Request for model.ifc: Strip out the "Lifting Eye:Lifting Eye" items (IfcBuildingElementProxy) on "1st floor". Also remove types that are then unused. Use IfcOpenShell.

First a look at what the model holds.

```python
import ifcopenshell
import ifcopenshell.util.element

model = ifcopenshell.open("model.ifc")
print(model.schema)
storey = next(s for s in model.by_type("IfcBuildingStorey") if s.Name == "1st floor")
proxies = [e for e in ifcopenshell.util.element.get_decomposition(storey) if e.is_a("IfcBuildingElementProxy")]
seen = {}
for e in proxies:
    element_type = ifcopenshell.util.element.get_type(e)
    name = element_type.Name if element_type not in (None, e) else None
    seen[name] = seen.get(name, 0) + 1
for name, count in sorted(seen.items(), key=str):
    print(count, "x", name)
```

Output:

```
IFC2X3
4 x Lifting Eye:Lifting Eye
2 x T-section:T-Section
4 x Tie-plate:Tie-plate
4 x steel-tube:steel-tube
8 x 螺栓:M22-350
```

```python
import ifcopenshell
import ifcopenshell.api.root
import ifcopenshell.util.element

model = ifcopenshell.open("model.ifc")

storey = next(s for s in model.by_type("IfcBuildingStorey") if s.Name == "1st floor")
proxies = [e for e in ifcopenshell.util.element.get_decomposition(storey) if e.is_a("IfcBuildingElementProxy")]
targets = [e for e in proxies if (t := ifcopenshell.util.element.get_type(e)) not in (None, e) and t.Name == "Lifting Eye:Lifting Eye"]
types = {ifcopenshell.util.element.get_type(e) for e in targets} - {None, *targets}

for e in targets:
    ifcopenshell.api.root.remove_product(model, product=e)
print(len(targets), "removed")

unused = [t for t in types if not ifcopenshell.util.element.get_types(t)]
for t in unused:
    ifcopenshell.api.root.remove_product(model, product=t)
print(len(unused), "unused types removed")

model.write("model_edited.ifc")
```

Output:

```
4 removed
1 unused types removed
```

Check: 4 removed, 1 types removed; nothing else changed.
